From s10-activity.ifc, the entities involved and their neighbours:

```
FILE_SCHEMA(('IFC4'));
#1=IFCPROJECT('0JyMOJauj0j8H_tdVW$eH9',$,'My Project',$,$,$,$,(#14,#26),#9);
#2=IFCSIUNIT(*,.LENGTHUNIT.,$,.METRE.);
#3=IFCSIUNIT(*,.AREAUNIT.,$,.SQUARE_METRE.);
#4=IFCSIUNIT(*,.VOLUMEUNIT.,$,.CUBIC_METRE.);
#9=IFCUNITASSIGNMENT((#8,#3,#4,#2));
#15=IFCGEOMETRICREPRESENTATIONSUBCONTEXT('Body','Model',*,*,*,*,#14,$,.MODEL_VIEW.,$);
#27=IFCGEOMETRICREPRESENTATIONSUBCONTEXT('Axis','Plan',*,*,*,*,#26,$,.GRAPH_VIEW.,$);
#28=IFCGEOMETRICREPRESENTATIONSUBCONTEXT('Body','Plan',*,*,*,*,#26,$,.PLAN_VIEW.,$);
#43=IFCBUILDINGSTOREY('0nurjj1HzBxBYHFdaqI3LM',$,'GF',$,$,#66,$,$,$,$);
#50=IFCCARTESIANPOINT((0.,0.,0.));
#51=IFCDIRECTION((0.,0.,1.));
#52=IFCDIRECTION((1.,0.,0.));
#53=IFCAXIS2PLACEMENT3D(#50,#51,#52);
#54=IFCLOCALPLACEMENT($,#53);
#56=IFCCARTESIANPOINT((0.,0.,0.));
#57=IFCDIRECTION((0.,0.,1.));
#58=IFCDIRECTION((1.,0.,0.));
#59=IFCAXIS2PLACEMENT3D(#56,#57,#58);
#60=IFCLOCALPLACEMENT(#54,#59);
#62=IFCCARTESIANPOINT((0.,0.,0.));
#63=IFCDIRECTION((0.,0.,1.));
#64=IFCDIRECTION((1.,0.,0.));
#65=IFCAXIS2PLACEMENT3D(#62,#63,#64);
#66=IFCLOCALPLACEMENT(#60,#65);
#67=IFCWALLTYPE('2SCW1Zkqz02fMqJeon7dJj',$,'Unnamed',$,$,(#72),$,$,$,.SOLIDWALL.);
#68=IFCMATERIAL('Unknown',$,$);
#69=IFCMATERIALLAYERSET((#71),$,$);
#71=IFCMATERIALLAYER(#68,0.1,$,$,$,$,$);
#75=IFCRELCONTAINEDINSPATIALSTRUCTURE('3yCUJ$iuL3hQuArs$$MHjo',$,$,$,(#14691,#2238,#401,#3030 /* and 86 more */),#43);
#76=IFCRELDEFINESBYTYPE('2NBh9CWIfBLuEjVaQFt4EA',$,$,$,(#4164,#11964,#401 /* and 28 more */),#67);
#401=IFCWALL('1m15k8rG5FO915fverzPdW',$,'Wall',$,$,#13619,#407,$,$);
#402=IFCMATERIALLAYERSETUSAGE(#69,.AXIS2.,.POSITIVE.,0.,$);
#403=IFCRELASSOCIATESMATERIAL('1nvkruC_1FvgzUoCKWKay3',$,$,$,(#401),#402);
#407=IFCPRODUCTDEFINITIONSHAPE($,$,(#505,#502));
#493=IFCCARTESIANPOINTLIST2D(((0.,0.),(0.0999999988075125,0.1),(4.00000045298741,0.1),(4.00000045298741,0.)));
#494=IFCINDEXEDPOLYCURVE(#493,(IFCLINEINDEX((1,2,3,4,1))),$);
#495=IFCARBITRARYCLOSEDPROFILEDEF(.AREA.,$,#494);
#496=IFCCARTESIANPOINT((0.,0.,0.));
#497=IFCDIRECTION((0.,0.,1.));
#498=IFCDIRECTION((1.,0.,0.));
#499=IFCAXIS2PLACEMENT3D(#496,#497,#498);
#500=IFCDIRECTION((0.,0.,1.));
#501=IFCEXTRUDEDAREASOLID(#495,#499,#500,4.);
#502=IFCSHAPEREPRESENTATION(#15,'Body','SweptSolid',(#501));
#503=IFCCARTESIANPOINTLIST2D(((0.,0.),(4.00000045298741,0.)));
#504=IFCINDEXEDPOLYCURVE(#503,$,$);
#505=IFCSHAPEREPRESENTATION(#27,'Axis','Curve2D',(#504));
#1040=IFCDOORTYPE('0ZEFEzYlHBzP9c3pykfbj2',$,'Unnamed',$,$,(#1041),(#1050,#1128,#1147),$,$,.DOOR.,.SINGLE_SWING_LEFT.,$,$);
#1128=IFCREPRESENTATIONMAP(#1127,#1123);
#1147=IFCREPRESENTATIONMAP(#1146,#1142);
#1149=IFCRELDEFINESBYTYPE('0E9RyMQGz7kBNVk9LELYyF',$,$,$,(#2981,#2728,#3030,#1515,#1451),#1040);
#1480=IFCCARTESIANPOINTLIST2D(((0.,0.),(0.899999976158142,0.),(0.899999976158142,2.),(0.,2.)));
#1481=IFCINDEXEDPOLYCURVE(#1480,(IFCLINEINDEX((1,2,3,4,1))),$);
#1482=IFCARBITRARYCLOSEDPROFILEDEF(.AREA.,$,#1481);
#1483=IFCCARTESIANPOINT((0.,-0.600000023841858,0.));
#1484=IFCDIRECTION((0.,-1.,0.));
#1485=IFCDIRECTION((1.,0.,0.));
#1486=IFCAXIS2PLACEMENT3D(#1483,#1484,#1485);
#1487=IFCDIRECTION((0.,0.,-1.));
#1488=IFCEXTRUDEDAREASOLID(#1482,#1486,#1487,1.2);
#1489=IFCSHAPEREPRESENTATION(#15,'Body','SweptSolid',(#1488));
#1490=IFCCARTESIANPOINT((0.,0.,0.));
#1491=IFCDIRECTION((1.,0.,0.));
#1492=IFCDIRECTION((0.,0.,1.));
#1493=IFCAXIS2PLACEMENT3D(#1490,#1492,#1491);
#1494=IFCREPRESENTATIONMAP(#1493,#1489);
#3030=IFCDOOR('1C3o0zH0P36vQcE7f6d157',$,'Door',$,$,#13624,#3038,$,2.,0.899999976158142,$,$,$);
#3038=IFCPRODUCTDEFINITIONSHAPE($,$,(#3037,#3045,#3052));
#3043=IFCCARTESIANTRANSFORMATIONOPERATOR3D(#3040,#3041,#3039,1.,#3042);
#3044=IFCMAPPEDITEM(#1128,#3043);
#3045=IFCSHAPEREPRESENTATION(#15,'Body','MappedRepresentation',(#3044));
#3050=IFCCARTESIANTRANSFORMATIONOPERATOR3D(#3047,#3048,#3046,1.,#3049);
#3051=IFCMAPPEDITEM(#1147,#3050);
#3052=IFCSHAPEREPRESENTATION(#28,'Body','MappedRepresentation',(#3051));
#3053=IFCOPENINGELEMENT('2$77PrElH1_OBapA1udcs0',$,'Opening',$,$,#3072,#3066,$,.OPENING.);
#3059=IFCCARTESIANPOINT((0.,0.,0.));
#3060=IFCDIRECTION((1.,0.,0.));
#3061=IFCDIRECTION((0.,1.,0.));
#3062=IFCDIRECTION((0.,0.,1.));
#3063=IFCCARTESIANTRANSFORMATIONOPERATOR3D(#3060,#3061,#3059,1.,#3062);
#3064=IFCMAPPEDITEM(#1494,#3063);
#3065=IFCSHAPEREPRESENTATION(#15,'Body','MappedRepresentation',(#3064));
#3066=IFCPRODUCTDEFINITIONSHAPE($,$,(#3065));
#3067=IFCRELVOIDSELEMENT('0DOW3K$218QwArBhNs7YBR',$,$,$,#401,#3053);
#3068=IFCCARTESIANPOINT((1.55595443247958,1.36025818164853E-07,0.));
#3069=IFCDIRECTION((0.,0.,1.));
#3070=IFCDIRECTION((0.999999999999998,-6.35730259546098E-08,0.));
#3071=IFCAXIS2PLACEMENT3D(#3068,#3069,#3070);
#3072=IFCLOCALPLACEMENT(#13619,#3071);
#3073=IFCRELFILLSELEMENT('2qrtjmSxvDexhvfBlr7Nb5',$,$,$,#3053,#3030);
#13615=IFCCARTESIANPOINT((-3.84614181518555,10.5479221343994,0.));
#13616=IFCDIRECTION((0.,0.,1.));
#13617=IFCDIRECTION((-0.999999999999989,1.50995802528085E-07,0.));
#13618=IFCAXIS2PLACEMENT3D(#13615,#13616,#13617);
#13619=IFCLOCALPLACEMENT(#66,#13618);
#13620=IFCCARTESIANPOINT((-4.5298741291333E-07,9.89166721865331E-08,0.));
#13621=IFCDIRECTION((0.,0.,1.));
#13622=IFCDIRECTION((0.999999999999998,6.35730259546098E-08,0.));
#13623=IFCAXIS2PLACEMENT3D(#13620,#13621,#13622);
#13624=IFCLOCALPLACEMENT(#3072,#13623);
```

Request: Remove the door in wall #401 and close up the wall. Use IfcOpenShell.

```python
import ifcopenshell
import ifcopenshell.api.feature
import ifcopenshell.api.root
import ifcopenshell.geom
import ifcopenshell.util.shape

model = ifcopenshell.open("s10-activity.ifc")
settings = ifcopenshell.geom.settings()


def volume(element):
    """Net volume in cubic metres, openings subtracted."""
    shape = ifcopenshell.geom.create_shape(settings, element)
    return ifcopenshell.util.shape.get_volume(shape.geometry)


door = model.by_id(3030)
opening = door.FillsVoids[0].RelatingOpeningElement
wall = opening.VoidsElements[0].RelatingBuildingElement
before = volume(wall)

ifcopenshell.api.root.remove_product(model, product=door)
ifcopenshell.api.feature.remove_feature(model, feature=opening)

after = volume(wall)

print(f"wall volume {before:.3f} -> {after:.3f} m3")

model.write("s10-activity_edited.ifc")
```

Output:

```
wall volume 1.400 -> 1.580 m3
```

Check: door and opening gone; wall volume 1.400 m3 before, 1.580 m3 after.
